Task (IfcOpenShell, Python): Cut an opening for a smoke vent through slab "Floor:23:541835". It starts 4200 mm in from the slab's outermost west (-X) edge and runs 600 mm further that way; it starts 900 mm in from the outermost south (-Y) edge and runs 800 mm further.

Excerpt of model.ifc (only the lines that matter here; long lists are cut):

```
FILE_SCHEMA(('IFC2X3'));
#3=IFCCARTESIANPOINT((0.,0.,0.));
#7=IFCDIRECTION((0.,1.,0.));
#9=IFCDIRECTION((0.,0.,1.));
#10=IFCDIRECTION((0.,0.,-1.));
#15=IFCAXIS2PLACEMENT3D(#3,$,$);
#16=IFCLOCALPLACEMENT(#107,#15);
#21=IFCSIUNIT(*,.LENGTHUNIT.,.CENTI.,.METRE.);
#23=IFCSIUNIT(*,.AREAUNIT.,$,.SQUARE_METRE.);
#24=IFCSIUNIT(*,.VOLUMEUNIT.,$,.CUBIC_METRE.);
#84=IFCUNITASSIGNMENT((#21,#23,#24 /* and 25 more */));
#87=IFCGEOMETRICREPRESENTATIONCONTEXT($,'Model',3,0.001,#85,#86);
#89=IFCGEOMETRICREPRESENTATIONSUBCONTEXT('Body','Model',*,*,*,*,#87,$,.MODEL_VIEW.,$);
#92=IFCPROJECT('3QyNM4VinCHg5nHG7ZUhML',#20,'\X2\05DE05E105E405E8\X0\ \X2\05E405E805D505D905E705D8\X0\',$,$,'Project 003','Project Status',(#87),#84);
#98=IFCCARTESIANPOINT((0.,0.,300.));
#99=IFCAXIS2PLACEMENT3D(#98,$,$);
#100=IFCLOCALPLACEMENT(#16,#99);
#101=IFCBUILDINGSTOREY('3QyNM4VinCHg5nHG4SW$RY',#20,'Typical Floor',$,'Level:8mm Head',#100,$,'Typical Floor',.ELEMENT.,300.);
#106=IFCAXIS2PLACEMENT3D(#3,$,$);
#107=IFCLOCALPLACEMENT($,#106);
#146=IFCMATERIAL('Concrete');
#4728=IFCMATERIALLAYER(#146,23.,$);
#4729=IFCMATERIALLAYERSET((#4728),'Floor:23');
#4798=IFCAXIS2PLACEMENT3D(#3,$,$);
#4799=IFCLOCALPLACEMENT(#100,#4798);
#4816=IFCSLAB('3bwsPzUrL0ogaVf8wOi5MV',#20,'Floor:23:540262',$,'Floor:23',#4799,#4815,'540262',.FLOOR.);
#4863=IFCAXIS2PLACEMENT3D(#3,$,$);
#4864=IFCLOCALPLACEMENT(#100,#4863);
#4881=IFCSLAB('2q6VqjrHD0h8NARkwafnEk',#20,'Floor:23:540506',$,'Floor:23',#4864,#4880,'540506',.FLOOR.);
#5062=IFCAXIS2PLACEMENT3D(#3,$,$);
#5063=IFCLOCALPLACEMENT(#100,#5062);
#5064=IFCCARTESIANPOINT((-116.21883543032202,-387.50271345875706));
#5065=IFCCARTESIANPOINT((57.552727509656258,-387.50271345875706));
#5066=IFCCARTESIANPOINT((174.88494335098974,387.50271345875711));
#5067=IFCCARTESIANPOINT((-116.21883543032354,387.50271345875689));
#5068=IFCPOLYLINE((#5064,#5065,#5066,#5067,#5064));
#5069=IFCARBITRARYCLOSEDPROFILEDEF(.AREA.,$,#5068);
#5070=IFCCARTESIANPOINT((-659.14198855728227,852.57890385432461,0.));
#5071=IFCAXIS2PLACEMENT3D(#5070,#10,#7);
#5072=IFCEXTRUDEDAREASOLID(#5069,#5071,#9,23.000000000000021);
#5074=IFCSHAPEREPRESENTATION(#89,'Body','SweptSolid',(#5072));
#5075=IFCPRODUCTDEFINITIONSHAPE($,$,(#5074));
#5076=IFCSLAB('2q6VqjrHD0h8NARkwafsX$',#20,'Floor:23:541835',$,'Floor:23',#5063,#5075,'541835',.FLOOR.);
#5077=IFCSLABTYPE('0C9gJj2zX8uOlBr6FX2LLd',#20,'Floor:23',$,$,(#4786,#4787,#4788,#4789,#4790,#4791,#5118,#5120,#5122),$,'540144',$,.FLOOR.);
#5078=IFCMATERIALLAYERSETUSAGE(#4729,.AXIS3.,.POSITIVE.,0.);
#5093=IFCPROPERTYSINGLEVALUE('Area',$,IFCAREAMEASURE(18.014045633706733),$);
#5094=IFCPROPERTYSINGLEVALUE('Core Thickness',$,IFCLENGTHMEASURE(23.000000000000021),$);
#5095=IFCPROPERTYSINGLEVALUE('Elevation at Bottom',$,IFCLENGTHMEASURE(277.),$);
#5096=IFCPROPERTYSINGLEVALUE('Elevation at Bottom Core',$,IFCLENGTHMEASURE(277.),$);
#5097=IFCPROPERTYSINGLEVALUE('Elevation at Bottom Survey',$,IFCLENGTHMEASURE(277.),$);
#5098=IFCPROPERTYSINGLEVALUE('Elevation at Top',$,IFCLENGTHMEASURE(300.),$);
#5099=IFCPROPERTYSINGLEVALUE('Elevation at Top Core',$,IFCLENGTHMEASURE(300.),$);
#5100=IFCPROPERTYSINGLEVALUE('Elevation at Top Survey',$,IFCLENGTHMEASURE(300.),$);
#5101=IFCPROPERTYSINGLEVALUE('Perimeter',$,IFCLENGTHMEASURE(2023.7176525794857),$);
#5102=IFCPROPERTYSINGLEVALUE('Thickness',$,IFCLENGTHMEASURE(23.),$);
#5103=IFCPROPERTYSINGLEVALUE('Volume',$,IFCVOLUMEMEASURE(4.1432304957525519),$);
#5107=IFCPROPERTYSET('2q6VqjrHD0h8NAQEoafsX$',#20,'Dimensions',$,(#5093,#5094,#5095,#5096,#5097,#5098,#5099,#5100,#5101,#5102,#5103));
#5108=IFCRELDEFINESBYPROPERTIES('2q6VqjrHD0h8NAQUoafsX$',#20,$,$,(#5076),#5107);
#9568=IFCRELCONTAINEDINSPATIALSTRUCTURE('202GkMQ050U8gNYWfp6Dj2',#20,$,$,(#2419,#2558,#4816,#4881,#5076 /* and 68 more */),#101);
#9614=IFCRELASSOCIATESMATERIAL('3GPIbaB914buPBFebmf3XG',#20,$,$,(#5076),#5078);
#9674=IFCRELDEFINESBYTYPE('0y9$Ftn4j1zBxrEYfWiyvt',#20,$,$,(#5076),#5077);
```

```python
import numpy as np
import ifcopenshell
import ifcopenshell.api.feature
import ifcopenshell.api.geometry
import ifcopenshell.api.pset
import ifcopenshell.api.root
import ifcopenshell.geom
import ifcopenshell.util.element
import ifcopenshell.util.placement
import ifcopenshell.util.representation
import ifcopenshell.util.shape
import ifcopenshell.util.unit

model = ifcopenshell.open("model.ifc")
unit_scale = ifcopenshell.util.unit.calculate_unit_scale(model)
area_scale = ifcopenshell.util.unit.calculate_unit_scale(model, "AREAUNIT")
volume_scale = ifcopenshell.util.unit.calculate_unit_scale(model, "VOLUMEUNIT")
settings = ifcopenshell.geom.settings()


def volume(element):
    """Net volume in cubic metres, openings subtracted."""
    shape = ifcopenshell.geom.create_shape(settings, element)
    return ifcopenshell.util.shape.get_volume(shape.geometry)


slab = model.by_id(5076)
before = volume(slab)

# Extent in the slab's own axes, in metres. The edges named are its -X and -Y sides.
slab_shape = ifcopenshell.geom.create_shape(settings, slab)
vertices = ifcopenshell.util.shape.get_vertices(slab_shape.geometry)
x_min, y_min, bottom = vertices.min(axis=0)
top = vertices[:, 2].max()

opening = ifcopenshell.api.root.create_entity(model, ifc_class="IfcOpeningElement", name="Smoke vent opening")
context = ifcopenshell.util.representation.get_context(model, "Model", "Body", "MODEL_VIEW")
width, depth = 0.6, 0.8
outline = [(0.0, 0.0), (width, 0.0), (width, depth), (0.0, depth), (0.0, 0.0)]
# Overshoot both faces by 50 mm so the cut is clean.
shape = ifcopenshell.api.geometry.add_slab_representation(
    model, context=context, depth=top - bottom + 0.1, polyline=outline
)
ifcopenshell.api.geometry.assign_representation(model, product=opening, representation=shape)

matrix = ifcopenshell.util.placement.get_local_placement(slab.ObjectPlacement)
matrix[:, 3] = matrix @ np.append(np.array([x_min + 4.2, y_min + 0.9, bottom - 0.05]) / unit_scale, 1.0)
ifcopenshell.api.geometry.edit_object_placement(model, product=opening, matrix=matrix, is_si=False)
ifcopenshell.api.feature.add_feature(model, feature=opening, element=slab)

after = volume(slab)

# Update the slab's stored quantities.
pset = model.by_id(ifcopenshell.util.element.get_pset(slab, "Dimensions", should_inherit=False)["id"])
ifcopenshell.api.pset.edit_pset(model, pset=pset, properties={
    "Area": model.create_entity("IfcAreaMeasure", after / (top - bottom) / area_scale),
    "Volume": model.create_entity("IfcVolumeMeasure", after / volume_scale),
})

print(f"slab volume {before:.3f} -> {after:.3f} m3")

model.write("model_edited.ifc")
```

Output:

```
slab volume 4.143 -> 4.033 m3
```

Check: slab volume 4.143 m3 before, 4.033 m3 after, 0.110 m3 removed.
